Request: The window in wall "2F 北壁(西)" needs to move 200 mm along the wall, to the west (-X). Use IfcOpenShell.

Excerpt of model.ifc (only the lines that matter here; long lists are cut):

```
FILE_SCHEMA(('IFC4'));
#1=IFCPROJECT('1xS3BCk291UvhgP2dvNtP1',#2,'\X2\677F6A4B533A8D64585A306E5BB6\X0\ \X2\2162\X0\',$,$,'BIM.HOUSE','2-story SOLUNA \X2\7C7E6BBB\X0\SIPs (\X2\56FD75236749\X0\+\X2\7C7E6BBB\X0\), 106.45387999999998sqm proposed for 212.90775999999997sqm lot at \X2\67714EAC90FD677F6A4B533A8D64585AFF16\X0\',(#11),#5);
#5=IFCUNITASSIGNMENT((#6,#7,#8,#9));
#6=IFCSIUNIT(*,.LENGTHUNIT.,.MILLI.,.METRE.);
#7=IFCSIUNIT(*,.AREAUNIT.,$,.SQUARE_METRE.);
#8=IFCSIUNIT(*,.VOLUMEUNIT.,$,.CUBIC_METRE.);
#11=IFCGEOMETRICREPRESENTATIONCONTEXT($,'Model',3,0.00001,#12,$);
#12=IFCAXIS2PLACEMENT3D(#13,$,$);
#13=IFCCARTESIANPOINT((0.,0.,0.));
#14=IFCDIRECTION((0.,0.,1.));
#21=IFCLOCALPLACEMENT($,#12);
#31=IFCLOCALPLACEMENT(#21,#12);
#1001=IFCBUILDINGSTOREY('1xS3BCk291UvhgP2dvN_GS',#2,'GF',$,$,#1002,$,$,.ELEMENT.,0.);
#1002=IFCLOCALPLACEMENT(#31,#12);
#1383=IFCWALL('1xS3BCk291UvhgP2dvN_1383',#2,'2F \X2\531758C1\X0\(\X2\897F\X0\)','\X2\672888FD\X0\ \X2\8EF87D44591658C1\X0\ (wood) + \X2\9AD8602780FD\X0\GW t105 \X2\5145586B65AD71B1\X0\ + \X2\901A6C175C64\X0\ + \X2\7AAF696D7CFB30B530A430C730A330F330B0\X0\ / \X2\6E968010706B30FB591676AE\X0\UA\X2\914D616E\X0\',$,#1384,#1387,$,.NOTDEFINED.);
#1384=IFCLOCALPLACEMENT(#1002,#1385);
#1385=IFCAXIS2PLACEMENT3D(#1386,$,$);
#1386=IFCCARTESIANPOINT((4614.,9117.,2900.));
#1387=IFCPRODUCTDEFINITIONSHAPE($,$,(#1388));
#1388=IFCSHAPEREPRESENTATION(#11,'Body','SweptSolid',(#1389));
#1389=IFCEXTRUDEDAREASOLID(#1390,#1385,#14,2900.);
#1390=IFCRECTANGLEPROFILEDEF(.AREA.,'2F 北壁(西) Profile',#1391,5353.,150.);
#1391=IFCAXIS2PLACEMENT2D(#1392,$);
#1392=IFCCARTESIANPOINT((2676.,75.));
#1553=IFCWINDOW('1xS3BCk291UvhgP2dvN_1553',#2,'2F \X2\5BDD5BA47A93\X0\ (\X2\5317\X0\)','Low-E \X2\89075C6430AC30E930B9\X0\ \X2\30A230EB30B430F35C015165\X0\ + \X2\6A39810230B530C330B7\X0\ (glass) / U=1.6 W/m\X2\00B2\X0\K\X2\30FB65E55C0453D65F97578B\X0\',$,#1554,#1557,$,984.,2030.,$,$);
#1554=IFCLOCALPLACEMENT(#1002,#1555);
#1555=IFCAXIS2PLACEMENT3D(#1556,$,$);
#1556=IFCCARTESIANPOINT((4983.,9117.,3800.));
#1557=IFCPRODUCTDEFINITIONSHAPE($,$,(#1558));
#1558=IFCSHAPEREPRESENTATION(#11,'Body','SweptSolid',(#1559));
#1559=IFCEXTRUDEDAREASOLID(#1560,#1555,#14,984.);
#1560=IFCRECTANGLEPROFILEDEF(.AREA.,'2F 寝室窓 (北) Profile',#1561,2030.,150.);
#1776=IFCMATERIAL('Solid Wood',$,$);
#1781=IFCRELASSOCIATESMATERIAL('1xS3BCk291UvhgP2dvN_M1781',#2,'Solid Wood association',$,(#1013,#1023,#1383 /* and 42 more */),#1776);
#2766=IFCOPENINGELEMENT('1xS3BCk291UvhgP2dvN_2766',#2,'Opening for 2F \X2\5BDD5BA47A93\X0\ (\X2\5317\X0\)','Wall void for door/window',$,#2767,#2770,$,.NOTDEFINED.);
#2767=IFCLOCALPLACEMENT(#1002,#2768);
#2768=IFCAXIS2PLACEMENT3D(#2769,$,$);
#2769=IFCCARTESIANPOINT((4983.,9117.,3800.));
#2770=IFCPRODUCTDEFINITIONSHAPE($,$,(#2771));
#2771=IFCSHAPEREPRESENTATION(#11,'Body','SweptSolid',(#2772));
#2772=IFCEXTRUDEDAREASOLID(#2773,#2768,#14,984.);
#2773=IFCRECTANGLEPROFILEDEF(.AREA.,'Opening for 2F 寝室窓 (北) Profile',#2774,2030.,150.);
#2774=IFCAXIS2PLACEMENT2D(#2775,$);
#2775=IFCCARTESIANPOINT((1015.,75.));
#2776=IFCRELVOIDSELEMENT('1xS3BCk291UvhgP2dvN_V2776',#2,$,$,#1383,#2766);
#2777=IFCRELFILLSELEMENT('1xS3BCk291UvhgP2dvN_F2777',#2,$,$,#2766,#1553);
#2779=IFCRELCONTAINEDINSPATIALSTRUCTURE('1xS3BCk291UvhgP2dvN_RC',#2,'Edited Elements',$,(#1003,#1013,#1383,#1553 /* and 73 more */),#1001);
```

```python
import ifcopenshell
import ifcopenshell.api.geometry
import ifcopenshell.util.placement
import ifcopenshell.util.unit

model = ifcopenshell.open("model.ifc")
unit_scale = ifcopenshell.util.unit.calculate_unit_scale(model)

window = model.by_guid("1xS3BCk291UvhgP2dvN_1553")
opening = window.FillsVoids[0].RelatingOpeningElement
wall = opening.VoidsElements[0].RelatingBuildingElement

wall_matrix = ifcopenshell.util.placement.get_local_placement(wall.ObjectPlacement)
shift = wall_matrix[:3, 0] * -0.2 / unit_scale
before = ifcopenshell.util.placement.get_local_placement(window.ObjectPlacement)[:3, 3].copy()

# The window is not placed relative to its opening, so move both.
for product in (opening, window):
    matrix = ifcopenshell.util.placement.get_local_placement(product.ObjectPlacement)
    matrix[:3, 3] += shift
    ifcopenshell.api.geometry.edit_object_placement(model, product=product, matrix=matrix, is_si=False)

after = ifcopenshell.util.placement.get_local_placement(window.ObjectPlacement)[:3, 3]
print("window moved by", (after - before).round(3) + 0.0)

model.write("model_edited.ifc")
```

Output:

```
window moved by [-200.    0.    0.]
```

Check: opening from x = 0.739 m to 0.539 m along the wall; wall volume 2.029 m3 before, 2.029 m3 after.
